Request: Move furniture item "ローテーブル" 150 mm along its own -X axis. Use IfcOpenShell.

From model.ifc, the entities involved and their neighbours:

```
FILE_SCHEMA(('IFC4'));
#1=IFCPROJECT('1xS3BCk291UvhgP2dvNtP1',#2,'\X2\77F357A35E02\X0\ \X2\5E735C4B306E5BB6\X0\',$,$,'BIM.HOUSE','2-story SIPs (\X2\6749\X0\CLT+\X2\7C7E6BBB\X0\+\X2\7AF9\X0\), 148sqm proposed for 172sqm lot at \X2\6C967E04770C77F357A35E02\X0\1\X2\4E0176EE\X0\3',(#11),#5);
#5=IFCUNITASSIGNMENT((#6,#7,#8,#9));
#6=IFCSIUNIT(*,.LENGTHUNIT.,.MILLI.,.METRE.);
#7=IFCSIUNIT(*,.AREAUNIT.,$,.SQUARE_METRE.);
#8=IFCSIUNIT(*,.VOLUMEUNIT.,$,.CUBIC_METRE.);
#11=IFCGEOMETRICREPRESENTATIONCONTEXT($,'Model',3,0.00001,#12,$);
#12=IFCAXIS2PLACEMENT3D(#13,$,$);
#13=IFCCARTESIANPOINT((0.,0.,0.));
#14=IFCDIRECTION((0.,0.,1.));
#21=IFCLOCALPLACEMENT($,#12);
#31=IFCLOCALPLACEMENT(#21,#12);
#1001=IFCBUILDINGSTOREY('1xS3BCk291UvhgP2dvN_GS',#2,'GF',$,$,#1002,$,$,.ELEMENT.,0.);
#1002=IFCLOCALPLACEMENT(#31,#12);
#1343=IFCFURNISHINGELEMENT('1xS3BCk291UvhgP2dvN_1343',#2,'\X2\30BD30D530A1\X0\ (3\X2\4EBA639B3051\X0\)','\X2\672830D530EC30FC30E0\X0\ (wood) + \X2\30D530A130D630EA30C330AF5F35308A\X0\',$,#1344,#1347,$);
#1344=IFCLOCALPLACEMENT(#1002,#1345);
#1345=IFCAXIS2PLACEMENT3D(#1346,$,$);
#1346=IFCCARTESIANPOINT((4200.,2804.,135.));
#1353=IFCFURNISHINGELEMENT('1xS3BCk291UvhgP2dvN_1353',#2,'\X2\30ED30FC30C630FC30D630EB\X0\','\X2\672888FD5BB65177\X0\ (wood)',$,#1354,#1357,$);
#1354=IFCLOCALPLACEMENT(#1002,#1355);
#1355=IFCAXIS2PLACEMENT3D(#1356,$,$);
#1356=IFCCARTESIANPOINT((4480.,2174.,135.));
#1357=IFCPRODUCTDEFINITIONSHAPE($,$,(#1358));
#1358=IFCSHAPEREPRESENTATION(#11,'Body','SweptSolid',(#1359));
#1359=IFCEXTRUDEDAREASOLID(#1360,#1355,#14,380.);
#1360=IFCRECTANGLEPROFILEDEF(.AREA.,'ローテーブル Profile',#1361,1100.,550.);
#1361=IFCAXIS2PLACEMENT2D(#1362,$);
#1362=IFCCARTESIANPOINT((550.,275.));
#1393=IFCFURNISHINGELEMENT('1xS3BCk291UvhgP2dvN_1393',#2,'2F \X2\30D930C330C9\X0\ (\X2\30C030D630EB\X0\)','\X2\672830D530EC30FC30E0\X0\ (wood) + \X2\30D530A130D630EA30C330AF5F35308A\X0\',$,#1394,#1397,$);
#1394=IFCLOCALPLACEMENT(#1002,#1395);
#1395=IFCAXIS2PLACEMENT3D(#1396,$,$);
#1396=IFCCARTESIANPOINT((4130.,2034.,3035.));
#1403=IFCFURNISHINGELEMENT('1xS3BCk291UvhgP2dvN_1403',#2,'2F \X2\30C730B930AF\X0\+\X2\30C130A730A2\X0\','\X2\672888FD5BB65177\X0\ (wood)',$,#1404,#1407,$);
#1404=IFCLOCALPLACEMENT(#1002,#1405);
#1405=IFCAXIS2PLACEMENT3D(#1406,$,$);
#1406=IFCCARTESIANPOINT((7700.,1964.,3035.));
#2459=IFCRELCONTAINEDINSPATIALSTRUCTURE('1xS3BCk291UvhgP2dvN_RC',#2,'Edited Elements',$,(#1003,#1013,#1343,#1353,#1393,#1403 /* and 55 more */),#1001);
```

```python
import ifcopenshell
import ifcopenshell.api.geometry
import ifcopenshell.util.placement
import ifcopenshell.util.unit

model = ifcopenshell.open("model.ifc")
unit_scale = ifcopenshell.util.unit.calculate_unit_scale(model)

item = model.by_guid("1xS3BCk291UvhgP2dvN_1353")
matrix = ifcopenshell.util.placement.get_local_placement(item.ObjectPlacement)
matrix[:3, 3] -= matrix[:3, 0] * 0.15 / unit_scale
ifcopenshell.api.geometry.edit_object_placement(model, product=item, matrix=matrix, is_si=False)

print(ifcopenshell.util.placement.get_local_placement(item.ObjectPlacement).round(3) + 0.0)

model.write("model_v2.ifc")
```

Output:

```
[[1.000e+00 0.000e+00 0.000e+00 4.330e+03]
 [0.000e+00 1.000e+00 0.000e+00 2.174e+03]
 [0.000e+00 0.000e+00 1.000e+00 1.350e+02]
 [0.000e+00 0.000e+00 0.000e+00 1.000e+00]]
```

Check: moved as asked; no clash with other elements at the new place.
